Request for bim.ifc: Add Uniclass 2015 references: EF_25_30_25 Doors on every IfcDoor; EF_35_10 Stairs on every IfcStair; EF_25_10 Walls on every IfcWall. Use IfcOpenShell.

First a look at what the model holds.

```python
import ifcopenshell

model = ifcopenshell.open("bim.ifc")
print(model.schema)
print("classifications:", [c.Name for c in model.by_type("IfcClassification")])
for ifc_class in ("IfcDoor", "IfcRoof", "IfcStair", "IfcWall", "IfcWindow"):
    print(ifc_class, len(model.by_type(ifc_class)))
```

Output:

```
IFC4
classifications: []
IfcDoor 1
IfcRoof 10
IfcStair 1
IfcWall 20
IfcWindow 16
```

```python
import ifcopenshell
import ifcopenshell.api.classification

model = ifcopenshell.open("bim.ifc")

system = ifcopenshell.api.classification.add_classification(model, classification="Uniclass 2015")

codes = {
    "IfcDoor": ("EF_25_30_25", "Doors"),
    "IfcStair": ("EF_35_10", "Stairs"),
    "IfcWall": ("EF_25_10", "Walls"),
}
for ifc_class, (code, name) in codes.items():
    products = model.by_type(ifc_class)
    ifcopenshell.api.classification.add_reference(
        model, products=products, classification=system, identification=code, name=name
    )
    print(code, len(products))

model.write("bim_v2.ifc")
```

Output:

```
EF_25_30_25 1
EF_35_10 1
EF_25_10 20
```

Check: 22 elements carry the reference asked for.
